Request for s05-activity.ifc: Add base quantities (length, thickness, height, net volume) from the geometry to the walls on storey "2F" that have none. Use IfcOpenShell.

First a look at what the model holds.

```python
import ifcopenshell
import ifcopenshell.util.element
import ifcopenshell.util.unit

model = ifcopenshell.open("s05-activity.ifc")
print(model.schema)
for unit_type in ("LENGTHUNIT", "AREAUNIT", "VOLUMEUNIT"):
    print(unit_type, ifcopenshell.util.unit.calculate_unit_scale(model, unit_type))
storey = next(s for s in model.by_type("IfcBuildingStorey") if s.Name == "2F")
walls = [e for e in ifcopenshell.util.element.get_decomposition(storey) if e.is_a("IfcWall")]
for e in sorted(walls, key=lambda e: e.id()):
    print(e.id(), e.is_a(), e.Name, list(ifcopenshell.util.element.get_psets(e, qtos_only=True)), sep=" | ")
```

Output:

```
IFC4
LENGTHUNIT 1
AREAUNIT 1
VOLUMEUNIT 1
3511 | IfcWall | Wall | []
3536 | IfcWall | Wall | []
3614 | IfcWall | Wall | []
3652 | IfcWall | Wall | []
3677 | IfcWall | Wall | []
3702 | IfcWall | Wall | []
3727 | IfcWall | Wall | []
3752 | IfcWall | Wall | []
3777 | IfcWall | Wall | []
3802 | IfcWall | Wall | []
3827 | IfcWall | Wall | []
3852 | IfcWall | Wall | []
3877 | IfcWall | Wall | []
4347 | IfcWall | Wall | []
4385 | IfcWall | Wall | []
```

```python
import ifcopenshell
import ifcopenshell.api.pset
import ifcopenshell.geom
import ifcopenshell.util.element
import ifcopenshell.util.shape
import ifcopenshell.util.unit

model = ifcopenshell.open("s05-activity.ifc")
unit_scale = ifcopenshell.util.unit.calculate_unit_scale(model)
volume_scale = ifcopenshell.util.unit.calculate_unit_scale(model, "VOLUMEUNIT")
settings = ifcopenshell.geom.settings()

storey = next(s for s in model.by_type("IfcBuildingStorey") if s.Name == "2F")
walls = [e for e in ifcopenshell.util.element.get_decomposition(storey) if e.is_a("IfcWall")]

for e in sorted(walls, key=lambda e: e.id()):
    if ifcopenshell.util.element.get_psets(e, qtos_only=True, should_inherit=False):
        continue
    # Geometry comes back in metres, in the element's own axes.
    shape = ifcopenshell.geom.create_shape(settings, e)
    values = {
        "Length": ifcopenshell.util.shape.get_x(shape.geometry) / unit_scale,
        "Width": ifcopenshell.util.shape.get_y(shape.geometry) / unit_scale,
        "Height": ifcopenshell.util.shape.get_z(shape.geometry) / unit_scale,
        "NetVolume": ifcopenshell.util.shape.get_volume(shape.geometry) / volume_scale,
    }
    qto = ifcopenshell.api.pset.add_qto(model, product=e, name="Qto_WallBaseQuantities")
    ifcopenshell.api.pset.edit_qto(model, qto=qto, properties=values)
    print(e.id(), {k: round(v, 3) for k, v in values.items()})

model.write("s05-activity_edited.ifc")
```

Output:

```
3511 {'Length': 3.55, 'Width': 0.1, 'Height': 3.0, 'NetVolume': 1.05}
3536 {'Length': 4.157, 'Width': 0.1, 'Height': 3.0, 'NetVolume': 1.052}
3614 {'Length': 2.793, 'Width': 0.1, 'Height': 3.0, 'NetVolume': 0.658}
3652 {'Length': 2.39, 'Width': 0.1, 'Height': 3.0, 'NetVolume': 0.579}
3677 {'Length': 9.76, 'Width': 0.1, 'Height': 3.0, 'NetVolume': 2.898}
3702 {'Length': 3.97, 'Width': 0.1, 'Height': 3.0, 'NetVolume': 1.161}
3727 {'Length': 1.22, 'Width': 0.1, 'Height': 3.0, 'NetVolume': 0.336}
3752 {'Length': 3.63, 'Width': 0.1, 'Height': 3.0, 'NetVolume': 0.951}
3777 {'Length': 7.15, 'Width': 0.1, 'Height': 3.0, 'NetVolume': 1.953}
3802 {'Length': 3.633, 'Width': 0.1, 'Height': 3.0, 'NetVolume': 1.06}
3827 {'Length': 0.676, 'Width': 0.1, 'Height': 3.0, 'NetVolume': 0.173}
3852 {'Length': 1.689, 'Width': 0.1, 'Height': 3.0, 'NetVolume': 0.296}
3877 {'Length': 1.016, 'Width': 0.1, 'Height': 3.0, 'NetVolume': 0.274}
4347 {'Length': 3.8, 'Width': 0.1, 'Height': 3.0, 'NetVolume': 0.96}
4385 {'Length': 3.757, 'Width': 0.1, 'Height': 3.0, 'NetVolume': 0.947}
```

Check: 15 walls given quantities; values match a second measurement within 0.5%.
